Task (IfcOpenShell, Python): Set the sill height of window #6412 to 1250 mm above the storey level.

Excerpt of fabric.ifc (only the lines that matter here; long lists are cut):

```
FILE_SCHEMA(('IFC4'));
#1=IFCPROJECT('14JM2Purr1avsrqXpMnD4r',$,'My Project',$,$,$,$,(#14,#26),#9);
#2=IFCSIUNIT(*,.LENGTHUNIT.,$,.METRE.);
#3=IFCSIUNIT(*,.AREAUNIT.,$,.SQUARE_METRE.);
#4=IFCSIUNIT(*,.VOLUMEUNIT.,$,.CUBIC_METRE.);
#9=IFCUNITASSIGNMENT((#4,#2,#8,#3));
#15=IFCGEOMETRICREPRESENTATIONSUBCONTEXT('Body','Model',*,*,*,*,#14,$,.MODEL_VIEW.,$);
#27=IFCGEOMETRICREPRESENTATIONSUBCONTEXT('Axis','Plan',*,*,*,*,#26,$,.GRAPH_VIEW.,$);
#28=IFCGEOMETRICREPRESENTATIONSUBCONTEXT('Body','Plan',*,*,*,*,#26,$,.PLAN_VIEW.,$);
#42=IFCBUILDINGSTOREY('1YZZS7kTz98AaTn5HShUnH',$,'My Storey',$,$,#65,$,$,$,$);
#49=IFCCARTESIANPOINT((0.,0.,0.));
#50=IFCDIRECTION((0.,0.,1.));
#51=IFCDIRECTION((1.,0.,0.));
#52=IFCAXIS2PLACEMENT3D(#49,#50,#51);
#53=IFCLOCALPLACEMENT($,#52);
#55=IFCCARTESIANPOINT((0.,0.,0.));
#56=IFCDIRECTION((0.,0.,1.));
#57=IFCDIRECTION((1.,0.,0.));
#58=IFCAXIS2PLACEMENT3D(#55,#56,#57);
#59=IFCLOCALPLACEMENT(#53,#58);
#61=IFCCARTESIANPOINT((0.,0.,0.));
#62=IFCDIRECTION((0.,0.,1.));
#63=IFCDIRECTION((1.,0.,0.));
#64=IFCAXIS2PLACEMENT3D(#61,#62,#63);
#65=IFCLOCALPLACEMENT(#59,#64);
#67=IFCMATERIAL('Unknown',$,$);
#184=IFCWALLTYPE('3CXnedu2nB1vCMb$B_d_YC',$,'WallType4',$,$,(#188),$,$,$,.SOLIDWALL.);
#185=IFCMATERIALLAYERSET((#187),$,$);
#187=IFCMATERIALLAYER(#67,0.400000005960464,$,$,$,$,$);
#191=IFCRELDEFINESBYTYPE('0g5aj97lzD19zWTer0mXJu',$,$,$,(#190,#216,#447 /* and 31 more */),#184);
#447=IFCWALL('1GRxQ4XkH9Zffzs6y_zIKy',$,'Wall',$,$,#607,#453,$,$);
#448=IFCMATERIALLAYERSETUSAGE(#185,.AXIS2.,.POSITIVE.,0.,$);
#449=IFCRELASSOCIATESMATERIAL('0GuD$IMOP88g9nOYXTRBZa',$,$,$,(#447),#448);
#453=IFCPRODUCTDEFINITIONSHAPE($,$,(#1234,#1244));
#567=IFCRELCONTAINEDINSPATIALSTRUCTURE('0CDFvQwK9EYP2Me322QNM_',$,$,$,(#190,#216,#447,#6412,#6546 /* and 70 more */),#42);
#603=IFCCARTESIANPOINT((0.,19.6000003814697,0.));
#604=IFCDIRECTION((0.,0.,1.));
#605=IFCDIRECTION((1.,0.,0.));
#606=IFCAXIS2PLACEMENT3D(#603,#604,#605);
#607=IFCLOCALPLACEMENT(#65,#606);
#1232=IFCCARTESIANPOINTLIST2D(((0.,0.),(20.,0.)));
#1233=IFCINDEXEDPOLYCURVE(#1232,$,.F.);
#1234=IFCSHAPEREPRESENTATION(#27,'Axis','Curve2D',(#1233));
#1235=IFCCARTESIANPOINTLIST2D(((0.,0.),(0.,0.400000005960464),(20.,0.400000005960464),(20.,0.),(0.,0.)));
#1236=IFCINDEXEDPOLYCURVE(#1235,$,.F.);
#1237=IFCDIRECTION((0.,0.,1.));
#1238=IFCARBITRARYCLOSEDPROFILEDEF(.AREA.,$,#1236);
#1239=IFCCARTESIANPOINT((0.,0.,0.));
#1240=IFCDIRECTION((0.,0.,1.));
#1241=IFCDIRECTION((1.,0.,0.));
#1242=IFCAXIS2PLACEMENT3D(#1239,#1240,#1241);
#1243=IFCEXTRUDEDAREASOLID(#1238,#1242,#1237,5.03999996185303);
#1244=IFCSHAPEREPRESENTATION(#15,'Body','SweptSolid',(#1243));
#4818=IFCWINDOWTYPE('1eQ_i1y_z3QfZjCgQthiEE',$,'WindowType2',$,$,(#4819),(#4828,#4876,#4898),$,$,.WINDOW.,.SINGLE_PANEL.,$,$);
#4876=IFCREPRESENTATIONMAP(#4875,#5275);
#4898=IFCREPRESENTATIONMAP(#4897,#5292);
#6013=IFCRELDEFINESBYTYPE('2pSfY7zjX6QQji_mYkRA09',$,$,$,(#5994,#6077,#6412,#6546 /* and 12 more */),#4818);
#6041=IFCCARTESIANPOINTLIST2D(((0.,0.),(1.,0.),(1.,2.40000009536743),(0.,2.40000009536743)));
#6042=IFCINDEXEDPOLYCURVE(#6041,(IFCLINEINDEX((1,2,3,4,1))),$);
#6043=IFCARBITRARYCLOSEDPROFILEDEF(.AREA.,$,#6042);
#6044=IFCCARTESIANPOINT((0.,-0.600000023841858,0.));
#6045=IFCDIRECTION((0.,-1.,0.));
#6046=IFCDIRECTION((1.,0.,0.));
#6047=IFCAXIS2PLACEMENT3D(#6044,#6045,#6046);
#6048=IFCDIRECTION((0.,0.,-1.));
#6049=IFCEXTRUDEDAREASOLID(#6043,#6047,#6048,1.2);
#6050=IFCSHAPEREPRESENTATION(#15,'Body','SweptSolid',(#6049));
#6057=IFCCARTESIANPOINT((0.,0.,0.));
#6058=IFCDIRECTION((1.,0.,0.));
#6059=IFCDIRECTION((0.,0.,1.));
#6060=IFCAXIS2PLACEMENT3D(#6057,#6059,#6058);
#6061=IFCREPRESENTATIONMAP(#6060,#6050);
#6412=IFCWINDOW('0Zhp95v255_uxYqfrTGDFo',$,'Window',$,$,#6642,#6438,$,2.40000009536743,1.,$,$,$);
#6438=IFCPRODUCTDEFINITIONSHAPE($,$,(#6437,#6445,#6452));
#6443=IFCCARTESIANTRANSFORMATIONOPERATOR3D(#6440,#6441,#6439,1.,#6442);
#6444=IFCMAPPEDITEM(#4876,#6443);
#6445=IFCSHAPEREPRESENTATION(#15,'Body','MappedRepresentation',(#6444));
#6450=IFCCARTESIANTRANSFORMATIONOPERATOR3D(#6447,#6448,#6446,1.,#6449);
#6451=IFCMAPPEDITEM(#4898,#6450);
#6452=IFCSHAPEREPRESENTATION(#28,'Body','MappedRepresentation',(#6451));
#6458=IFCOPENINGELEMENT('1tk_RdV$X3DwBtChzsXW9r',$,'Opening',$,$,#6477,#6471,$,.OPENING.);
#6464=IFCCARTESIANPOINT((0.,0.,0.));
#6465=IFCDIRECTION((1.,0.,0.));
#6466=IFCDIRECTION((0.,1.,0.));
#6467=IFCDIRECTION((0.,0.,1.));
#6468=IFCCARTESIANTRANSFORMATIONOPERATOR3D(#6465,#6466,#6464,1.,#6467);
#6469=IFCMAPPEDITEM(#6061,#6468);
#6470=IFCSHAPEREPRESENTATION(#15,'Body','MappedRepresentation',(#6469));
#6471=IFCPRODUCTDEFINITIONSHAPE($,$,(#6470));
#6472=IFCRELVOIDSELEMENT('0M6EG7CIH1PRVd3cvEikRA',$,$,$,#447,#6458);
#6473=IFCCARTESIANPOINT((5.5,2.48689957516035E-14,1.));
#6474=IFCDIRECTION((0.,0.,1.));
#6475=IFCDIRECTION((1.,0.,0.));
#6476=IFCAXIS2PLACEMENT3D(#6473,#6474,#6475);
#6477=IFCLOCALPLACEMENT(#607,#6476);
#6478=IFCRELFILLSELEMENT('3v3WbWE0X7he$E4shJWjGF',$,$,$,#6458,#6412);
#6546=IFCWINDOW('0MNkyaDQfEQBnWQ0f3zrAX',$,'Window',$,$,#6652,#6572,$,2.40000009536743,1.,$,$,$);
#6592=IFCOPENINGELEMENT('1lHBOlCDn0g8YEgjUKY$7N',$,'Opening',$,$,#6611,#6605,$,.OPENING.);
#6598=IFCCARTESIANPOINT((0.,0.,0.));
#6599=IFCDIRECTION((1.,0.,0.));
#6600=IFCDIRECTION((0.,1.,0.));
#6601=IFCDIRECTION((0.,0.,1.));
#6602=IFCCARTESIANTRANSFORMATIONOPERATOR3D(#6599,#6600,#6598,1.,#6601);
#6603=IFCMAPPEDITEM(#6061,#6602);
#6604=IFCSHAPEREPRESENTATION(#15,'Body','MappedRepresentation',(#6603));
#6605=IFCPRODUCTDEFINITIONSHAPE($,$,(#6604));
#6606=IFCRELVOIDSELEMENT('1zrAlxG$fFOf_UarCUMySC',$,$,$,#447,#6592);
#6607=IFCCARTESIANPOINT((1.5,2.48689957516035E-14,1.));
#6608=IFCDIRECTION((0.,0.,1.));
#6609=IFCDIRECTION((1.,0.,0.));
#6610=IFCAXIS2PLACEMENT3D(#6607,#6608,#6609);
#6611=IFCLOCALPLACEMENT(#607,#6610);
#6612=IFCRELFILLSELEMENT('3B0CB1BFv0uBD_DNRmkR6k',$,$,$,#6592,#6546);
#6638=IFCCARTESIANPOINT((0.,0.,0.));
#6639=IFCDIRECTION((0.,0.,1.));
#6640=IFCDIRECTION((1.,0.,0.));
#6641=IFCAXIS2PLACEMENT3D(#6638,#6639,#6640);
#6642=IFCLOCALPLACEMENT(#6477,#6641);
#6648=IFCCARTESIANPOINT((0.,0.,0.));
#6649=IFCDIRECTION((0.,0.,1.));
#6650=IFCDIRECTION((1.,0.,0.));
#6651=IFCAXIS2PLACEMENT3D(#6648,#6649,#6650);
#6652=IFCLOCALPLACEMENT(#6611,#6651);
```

```python
import numpy as np
import ifcopenshell
import ifcopenshell.api.geometry
import ifcopenshell.geom
import ifcopenshell.util.element
import ifcopenshell.util.placement
import ifcopenshell.util.shape
import ifcopenshell.util.unit

model = ifcopenshell.open("fabric.ifc")
unit_scale = ifcopenshell.util.unit.calculate_unit_scale(model)

window = model.by_guid("0Zhp95v255_uxYqfrTGDFo")
opening = window.FillsVoids[0].RelatingOpeningElement
storey = ifcopenshell.util.element.get_container(window, ifc_class="IfcBuildingStorey")
level = ifcopenshell.util.placement.get_local_placement(storey.ObjectPlacement)[2, 3]

# The opening's origin need not be at the sill, so measure its lowest point.
shape = ifcopenshell.geom.create_shape(ifcopenshell.geom.settings(), opening)
bottom = ifcopenshell.util.shape.get_shape_bottom_elevation(shape, shape.geometry) / unit_scale
dz = level + 1.25 - bottom

shift = np.array([0.0, 0.0, dz])
# The window is placed relative to its opening, so it follows when the opening moves.
matrix = ifcopenshell.util.placement.get_local_placement(opening.ObjectPlacement)
matrix[:3, 3] += shift
ifcopenshell.api.geometry.edit_object_placement(
    model, product=opening, matrix=matrix, is_si=False, should_transform_children=True
)

print(f"moved by {dz * unit_scale:+.3f} m")

model.write("fabric_rev.ifc")
```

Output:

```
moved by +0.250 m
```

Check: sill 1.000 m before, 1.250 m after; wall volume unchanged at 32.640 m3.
